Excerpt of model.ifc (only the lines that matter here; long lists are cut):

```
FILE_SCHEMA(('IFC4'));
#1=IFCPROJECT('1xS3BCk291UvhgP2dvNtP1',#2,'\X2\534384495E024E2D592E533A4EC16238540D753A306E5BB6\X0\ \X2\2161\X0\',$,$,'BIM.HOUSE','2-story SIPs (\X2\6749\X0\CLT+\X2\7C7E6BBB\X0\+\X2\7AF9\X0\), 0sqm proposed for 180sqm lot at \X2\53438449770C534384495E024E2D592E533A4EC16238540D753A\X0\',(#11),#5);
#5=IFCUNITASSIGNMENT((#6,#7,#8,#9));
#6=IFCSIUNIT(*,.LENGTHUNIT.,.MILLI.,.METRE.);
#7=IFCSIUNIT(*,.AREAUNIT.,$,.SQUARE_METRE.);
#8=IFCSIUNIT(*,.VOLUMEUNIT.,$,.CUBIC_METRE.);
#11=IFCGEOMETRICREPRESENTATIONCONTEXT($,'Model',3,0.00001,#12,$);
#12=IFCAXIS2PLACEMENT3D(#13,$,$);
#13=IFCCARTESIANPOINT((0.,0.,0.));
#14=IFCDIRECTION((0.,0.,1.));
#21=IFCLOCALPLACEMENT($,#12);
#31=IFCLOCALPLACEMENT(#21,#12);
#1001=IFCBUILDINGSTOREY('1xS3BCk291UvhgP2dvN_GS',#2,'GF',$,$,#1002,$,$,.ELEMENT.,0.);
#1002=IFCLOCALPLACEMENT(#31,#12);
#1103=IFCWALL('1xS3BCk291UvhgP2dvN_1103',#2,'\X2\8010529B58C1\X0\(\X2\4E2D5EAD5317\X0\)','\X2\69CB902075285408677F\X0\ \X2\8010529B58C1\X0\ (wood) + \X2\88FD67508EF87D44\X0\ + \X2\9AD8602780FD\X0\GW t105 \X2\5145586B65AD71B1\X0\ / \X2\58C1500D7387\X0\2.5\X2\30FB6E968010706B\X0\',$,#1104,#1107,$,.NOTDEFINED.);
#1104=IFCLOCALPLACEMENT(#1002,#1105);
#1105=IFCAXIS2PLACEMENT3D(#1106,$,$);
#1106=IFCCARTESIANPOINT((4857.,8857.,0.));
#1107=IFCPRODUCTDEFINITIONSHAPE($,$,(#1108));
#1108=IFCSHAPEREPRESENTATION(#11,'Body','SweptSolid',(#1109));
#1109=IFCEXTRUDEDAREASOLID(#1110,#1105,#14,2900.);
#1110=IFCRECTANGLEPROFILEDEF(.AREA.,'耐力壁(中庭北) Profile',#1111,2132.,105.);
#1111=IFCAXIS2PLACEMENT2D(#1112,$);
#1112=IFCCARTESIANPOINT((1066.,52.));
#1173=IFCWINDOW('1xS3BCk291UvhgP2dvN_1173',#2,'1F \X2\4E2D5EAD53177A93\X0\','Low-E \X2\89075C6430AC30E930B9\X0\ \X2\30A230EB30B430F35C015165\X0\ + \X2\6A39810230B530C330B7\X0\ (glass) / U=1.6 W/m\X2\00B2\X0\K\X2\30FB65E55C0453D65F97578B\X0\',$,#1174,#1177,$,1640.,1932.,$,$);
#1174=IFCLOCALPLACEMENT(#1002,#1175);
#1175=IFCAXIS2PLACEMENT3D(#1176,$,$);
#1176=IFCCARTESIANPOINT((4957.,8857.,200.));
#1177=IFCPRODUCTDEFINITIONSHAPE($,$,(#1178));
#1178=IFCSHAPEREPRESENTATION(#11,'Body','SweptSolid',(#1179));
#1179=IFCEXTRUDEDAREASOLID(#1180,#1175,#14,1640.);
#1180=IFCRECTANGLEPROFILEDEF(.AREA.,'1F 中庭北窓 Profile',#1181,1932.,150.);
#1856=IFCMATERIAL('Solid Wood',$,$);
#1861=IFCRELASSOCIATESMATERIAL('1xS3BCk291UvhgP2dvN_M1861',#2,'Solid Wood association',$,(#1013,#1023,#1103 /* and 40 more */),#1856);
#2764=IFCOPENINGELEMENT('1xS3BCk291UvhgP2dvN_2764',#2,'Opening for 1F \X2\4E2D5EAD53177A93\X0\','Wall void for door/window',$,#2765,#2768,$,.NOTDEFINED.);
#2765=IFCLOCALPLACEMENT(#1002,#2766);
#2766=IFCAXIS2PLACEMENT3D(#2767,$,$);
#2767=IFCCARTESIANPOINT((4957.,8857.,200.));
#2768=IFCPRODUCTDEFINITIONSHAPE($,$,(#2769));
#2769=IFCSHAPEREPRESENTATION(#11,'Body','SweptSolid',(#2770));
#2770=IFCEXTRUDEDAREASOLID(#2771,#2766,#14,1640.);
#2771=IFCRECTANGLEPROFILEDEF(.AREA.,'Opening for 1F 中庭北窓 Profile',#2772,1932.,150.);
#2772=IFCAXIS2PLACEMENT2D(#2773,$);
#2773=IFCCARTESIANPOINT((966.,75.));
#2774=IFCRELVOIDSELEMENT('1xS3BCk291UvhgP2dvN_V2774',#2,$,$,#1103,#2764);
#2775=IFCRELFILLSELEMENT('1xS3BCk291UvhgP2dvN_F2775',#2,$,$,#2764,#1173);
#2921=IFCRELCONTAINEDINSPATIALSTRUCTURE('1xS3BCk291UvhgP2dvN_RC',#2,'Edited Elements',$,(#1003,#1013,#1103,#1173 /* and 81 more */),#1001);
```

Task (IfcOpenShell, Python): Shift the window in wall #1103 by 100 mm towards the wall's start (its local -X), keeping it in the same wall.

```python
import ifcopenshell
import ifcopenshell.api.geometry
import ifcopenshell.util.placement

model = ifcopenshell.open("model.ifc")

window = model.by_id(1173)
opening = window.FillsVoids[0].RelatingOpeningElement
wall = opening.VoidsElements[0].RelatingBuildingElement

wall_matrix = ifcopenshell.util.placement.get_local_placement(wall.ObjectPlacement)
shift = wall_matrix[:3, 0] * -100.0
before = ifcopenshell.util.placement.get_local_placement(window.ObjectPlacement)[:3, 3].copy()

# The window is not placed relative to its opening, so move both.
for product in (opening, window):
    matrix = ifcopenshell.util.placement.get_local_placement(product.ObjectPlacement)
    matrix[:3, 3] += shift
    ifcopenshell.api.geometry.edit_object_placement(model, product=product, matrix=matrix, is_si=False)

after = ifcopenshell.util.placement.get_local_placement(window.ObjectPlacement)[:3, 3]
print("window moved by", (after - before).round(3) + 0.0)

model.write("model-out.ifc")
```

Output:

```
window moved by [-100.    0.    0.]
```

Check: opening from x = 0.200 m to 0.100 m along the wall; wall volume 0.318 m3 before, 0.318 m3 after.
